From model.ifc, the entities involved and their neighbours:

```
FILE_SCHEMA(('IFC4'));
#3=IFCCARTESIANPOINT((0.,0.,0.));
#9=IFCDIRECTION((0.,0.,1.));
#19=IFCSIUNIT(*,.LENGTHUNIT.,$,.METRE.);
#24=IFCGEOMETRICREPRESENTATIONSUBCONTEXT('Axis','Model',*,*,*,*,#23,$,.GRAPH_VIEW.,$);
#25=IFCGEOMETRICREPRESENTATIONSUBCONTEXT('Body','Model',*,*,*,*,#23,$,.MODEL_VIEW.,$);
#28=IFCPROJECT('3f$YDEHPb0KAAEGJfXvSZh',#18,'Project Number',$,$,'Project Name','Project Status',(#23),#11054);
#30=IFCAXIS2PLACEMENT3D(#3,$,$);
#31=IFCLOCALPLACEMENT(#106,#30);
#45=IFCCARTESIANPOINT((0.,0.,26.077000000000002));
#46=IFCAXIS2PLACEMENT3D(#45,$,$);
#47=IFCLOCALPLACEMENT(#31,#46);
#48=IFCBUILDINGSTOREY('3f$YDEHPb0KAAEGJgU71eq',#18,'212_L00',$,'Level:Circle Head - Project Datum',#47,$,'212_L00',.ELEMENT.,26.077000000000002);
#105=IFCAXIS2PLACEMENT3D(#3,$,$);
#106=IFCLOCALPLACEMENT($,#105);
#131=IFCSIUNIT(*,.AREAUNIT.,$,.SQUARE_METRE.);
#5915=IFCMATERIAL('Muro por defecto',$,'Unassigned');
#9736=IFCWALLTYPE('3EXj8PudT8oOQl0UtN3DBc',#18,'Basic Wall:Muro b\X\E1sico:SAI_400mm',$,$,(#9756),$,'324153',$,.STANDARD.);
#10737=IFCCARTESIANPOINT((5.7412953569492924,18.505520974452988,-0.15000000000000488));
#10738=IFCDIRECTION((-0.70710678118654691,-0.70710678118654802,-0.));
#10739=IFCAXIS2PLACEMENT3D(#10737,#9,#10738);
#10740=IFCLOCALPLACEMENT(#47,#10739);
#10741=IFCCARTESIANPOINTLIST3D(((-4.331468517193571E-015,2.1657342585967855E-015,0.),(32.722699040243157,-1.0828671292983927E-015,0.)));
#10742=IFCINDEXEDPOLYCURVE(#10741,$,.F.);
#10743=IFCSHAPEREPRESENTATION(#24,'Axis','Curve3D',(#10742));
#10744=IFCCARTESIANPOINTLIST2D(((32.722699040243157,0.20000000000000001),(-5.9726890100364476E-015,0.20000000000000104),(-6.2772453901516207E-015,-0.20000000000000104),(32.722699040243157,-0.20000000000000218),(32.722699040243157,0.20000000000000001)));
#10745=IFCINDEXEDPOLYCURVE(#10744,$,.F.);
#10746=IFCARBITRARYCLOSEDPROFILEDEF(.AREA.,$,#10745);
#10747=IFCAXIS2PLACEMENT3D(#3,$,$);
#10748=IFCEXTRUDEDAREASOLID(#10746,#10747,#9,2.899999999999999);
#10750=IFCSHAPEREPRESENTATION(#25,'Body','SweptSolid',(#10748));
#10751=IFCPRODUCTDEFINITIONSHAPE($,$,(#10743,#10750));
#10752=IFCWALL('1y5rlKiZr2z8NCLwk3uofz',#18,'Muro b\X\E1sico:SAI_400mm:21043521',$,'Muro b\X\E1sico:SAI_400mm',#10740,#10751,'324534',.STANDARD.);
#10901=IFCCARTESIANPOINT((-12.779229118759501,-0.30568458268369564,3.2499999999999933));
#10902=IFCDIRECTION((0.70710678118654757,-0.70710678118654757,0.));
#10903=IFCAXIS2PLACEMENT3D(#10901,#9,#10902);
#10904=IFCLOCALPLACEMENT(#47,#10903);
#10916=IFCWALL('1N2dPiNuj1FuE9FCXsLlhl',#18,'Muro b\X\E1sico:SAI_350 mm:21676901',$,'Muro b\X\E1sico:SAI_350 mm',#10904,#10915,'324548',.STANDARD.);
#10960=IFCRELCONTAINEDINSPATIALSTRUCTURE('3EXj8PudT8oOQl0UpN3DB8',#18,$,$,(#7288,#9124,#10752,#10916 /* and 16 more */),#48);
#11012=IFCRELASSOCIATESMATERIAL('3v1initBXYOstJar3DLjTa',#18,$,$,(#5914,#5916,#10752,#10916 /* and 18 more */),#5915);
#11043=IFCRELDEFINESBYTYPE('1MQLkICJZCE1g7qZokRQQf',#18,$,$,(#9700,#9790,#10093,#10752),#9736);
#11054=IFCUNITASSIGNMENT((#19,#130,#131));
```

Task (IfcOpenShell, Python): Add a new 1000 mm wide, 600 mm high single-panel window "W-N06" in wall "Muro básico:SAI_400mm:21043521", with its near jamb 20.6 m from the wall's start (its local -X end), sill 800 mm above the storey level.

```python
import numpy as np
import ifcopenshell
import ifcopenshell.api.feature
import ifcopenshell.api.geometry
import ifcopenshell.api.root
import ifcopenshell.api.spatial
import ifcopenshell.geom
import ifcopenshell.util.element
import ifcopenshell.util.placement
import ifcopenshell.util.representation
import ifcopenshell.util.shape
import ifcopenshell.util.unit

model = ifcopenshell.open("model.ifc")
unit_scale = ifcopenshell.util.unit.calculate_unit_scale(model)
settings = ifcopenshell.geom.settings()


def volume(element):
    """Net volume in cubic metres, openings subtracted."""
    shape = ifcopenshell.geom.create_shape(settings, element)
    return ifcopenshell.util.shape.get_volume(shape.geometry)


wall = model.by_id(10752)
storey = ifcopenshell.util.element.get_container(wall, ifc_class="IfcBuildingStorey")
context = ifcopenshell.util.representation.get_context(model, "Model", "Body", "MODEL_VIEW")
before = volume(wall)

width, height, from_end, sill = 1, 0.6, 20.6, 0.8  # metres

# The wall runs along its own X axis, and the end named is its -X end.
wall_shape = ifcopenshell.geom.create_shape(settings, wall)
x, y, z = ifcopenshell.util.shape.get_vertices(wall_shape.geometry).T
start = x.min() + from_end
face, thickness = float(y.min()), float(y.max() - y.min())
wall_matrix = ifcopenshell.util.placement.get_local_placement(wall.ObjectPlacement)
level = ifcopenshell.util.placement.get_local_placement(storey.ObjectPlacement)[2, 3]


def in_wall(x, y):
    """Placement at x, y metres in the wall's axes, at sill height."""
    matrix = wall_matrix.copy()
    matrix[:, 3] = wall_matrix @ np.array([x / unit_scale, y / unit_scale, 0.0, 1.0])
    matrix[2, 3] = level + sill / unit_scale
    return matrix


# Opening: a box that overshoots both wall faces by 50 mm.
opening = ifcopenshell.api.root.create_entity(model, ifc_class="IfcOpeningElement", predefined_type="OPENING")
box = ifcopenshell.api.geometry.add_wall_representation(
    model, context=context, length=width, height=height, thickness=thickness + 0.1
)
ifcopenshell.api.geometry.assign_representation(model, product=opening, representation=box)
ifcopenshell.api.geometry.edit_object_placement(model, product=opening, matrix=in_wall(start, face - 0.05), is_si=False)
ifcopenshell.api.feature.add_feature(model, feature=opening, element=wall)

window = ifcopenshell.api.root.create_entity(model, ifc_class="IfcWindow", name="W-N06", predefined_type="WINDOW")
window.OverallWidth, window.OverallHeight = width / unit_scale, height / unit_scale
window.PartitioningType = "SINGLE_PANEL"
body = ifcopenshell.api.geometry.add_window_representation(
    model,
    context=context,
    overall_width=window.OverallWidth,
    overall_height=window.OverallHeight,
    partition_type="SINGLE_PANEL",
)
ifcopenshell.api.geometry.assign_representation(model, product=window, representation=body)
ifcopenshell.api.spatial.assign_container(model, products=[window], relating_structure=storey)
ifcopenshell.api.feature.add_filling(model, opening=opening, element=window)

# Centre the window in the wall's thickness.
ifcopenshell.api.geometry.edit_object_placement(model, product=window, matrix=in_wall(start, face), is_si=False)
window_shape = ifcopenshell.geom.create_shape(settings, window)
depth = ifcopenshell.util.shape.get_vertices(window_shape.geometry)[:, 1]
offset = face + thickness / 2 - (depth.min() + depth.max()) / 2
ifcopenshell.api.geometry.edit_object_placement(model, product=window, matrix=in_wall(start, offset), is_si=False)

after = volume(wall)

print(f"wall volume {before:.3f} -> {after:.3f} m3")

model.write("model_edited.ifc")
```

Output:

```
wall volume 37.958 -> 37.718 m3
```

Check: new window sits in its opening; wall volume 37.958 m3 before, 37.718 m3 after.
